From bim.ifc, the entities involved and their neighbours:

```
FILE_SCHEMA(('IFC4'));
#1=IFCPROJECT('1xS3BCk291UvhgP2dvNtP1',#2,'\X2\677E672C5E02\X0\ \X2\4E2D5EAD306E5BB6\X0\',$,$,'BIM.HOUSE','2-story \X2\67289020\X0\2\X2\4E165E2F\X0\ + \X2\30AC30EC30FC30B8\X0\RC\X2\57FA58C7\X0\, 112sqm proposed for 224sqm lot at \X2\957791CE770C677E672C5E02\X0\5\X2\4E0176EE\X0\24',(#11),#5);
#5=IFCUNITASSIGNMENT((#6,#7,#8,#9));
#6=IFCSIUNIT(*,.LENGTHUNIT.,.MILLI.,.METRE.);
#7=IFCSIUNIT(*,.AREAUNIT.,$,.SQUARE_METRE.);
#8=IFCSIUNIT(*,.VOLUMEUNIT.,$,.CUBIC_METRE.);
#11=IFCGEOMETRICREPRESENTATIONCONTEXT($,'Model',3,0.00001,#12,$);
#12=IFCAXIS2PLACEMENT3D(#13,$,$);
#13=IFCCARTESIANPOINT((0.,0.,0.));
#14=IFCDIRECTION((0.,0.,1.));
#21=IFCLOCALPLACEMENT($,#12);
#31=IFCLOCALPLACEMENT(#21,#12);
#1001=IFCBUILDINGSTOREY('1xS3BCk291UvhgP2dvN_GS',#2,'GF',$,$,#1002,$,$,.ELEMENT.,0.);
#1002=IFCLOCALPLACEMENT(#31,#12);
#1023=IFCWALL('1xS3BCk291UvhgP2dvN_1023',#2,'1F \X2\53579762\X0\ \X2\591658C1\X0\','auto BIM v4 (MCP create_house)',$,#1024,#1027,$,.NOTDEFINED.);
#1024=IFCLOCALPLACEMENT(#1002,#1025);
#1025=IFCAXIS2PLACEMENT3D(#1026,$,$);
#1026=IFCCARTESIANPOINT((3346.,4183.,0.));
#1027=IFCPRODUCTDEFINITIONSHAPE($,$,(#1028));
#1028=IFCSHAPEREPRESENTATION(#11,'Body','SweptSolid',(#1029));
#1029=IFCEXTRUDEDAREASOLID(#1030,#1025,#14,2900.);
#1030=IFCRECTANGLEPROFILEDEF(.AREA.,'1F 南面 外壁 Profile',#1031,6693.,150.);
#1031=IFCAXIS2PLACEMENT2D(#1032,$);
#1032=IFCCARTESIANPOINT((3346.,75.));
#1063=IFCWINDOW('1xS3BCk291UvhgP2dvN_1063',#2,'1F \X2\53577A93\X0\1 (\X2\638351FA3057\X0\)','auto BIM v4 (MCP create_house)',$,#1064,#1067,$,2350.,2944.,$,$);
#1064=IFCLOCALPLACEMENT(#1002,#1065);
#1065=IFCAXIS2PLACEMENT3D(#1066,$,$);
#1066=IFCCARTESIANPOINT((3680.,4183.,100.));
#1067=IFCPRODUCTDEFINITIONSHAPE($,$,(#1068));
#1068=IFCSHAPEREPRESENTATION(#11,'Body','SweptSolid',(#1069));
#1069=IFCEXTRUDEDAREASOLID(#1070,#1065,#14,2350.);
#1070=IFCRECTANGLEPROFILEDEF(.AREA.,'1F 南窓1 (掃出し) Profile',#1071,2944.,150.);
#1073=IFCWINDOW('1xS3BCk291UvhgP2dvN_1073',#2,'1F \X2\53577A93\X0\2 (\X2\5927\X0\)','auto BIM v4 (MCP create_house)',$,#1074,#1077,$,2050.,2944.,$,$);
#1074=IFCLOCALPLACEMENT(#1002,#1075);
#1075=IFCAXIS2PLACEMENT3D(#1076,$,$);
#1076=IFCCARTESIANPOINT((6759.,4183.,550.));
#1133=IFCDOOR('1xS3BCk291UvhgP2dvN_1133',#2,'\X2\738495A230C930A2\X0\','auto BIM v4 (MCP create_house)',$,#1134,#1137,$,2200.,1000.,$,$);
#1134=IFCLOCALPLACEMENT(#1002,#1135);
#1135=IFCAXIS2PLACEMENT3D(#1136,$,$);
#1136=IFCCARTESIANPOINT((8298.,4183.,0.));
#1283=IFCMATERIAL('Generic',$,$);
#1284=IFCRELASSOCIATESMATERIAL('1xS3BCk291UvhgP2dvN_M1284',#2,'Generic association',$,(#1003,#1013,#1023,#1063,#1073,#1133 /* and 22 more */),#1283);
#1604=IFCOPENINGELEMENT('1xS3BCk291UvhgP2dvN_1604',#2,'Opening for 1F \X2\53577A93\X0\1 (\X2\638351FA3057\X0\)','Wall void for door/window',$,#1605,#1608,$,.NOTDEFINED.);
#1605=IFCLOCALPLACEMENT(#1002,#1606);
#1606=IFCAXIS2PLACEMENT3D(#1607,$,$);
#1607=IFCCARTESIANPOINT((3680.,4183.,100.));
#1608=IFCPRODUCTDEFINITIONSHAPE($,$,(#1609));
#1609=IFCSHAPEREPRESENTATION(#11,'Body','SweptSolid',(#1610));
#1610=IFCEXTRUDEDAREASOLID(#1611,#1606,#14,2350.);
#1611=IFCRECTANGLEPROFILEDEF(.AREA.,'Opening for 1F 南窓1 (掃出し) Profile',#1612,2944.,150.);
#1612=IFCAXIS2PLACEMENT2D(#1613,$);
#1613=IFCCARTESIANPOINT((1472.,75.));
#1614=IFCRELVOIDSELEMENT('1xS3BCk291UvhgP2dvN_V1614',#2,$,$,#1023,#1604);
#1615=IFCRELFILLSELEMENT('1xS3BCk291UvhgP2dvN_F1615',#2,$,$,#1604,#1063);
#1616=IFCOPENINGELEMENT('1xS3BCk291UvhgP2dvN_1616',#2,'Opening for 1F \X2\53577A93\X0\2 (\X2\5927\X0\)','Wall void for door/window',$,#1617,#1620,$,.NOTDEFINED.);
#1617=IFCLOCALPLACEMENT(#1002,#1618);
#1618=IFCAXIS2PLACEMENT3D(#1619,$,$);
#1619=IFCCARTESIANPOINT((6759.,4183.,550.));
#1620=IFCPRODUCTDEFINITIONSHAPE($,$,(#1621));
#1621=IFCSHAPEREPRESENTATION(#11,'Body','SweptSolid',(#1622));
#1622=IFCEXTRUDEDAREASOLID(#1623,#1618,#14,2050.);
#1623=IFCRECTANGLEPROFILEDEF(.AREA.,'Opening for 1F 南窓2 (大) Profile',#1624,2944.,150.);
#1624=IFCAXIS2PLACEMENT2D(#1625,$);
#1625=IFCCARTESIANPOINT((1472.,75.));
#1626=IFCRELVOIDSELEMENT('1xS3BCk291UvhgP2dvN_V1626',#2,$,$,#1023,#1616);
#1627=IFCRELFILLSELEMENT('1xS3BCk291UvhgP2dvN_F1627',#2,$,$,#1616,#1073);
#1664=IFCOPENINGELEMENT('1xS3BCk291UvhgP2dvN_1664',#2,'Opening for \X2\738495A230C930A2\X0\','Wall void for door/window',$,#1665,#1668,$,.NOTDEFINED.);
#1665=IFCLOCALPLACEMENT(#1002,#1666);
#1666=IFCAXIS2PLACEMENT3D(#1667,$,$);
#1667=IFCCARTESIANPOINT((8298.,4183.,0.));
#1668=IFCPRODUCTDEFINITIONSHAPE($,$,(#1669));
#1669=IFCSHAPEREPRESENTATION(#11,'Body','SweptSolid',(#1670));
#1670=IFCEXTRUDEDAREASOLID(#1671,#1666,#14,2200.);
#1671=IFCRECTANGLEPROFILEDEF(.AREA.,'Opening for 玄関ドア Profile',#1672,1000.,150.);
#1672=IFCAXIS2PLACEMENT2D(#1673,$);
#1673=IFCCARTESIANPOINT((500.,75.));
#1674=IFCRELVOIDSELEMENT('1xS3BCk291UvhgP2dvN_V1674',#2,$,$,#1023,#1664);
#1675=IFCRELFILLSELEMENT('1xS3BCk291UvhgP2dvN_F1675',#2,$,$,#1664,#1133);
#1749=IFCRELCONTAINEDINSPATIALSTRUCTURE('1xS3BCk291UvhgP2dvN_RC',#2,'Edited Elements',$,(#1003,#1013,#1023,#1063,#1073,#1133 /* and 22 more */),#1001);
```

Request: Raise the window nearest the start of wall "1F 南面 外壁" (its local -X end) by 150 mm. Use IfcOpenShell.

```python
import numpy as np
import ifcopenshell
import ifcopenshell.api.geometry
import ifcopenshell.util.placement
import ifcopenshell.util.unit

model = ifcopenshell.open("bim.ifc")
unit_scale = ifcopenshell.util.unit.calculate_unit_scale(model)

window = model.by_guid("1xS3BCk291UvhgP2dvN_1063")
opening = window.FillsVoids[0].RelatingOpeningElement
dz = 0.15 / unit_scale

shift = np.array([0.0, 0.0, dz])
# The window is not placed relative to its opening, so move both.
for product in (opening, window):
    matrix = ifcopenshell.util.placement.get_local_placement(product.ObjectPlacement)
    matrix[:3, 3] += shift
    ifcopenshell.api.geometry.edit_object_placement(model, product=product, matrix=matrix, is_si=False)

print(f"moved by {dz * unit_scale:+.3f} m")

model.write("bim-out.ifc")
```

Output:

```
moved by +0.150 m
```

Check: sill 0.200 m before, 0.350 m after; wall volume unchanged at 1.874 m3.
